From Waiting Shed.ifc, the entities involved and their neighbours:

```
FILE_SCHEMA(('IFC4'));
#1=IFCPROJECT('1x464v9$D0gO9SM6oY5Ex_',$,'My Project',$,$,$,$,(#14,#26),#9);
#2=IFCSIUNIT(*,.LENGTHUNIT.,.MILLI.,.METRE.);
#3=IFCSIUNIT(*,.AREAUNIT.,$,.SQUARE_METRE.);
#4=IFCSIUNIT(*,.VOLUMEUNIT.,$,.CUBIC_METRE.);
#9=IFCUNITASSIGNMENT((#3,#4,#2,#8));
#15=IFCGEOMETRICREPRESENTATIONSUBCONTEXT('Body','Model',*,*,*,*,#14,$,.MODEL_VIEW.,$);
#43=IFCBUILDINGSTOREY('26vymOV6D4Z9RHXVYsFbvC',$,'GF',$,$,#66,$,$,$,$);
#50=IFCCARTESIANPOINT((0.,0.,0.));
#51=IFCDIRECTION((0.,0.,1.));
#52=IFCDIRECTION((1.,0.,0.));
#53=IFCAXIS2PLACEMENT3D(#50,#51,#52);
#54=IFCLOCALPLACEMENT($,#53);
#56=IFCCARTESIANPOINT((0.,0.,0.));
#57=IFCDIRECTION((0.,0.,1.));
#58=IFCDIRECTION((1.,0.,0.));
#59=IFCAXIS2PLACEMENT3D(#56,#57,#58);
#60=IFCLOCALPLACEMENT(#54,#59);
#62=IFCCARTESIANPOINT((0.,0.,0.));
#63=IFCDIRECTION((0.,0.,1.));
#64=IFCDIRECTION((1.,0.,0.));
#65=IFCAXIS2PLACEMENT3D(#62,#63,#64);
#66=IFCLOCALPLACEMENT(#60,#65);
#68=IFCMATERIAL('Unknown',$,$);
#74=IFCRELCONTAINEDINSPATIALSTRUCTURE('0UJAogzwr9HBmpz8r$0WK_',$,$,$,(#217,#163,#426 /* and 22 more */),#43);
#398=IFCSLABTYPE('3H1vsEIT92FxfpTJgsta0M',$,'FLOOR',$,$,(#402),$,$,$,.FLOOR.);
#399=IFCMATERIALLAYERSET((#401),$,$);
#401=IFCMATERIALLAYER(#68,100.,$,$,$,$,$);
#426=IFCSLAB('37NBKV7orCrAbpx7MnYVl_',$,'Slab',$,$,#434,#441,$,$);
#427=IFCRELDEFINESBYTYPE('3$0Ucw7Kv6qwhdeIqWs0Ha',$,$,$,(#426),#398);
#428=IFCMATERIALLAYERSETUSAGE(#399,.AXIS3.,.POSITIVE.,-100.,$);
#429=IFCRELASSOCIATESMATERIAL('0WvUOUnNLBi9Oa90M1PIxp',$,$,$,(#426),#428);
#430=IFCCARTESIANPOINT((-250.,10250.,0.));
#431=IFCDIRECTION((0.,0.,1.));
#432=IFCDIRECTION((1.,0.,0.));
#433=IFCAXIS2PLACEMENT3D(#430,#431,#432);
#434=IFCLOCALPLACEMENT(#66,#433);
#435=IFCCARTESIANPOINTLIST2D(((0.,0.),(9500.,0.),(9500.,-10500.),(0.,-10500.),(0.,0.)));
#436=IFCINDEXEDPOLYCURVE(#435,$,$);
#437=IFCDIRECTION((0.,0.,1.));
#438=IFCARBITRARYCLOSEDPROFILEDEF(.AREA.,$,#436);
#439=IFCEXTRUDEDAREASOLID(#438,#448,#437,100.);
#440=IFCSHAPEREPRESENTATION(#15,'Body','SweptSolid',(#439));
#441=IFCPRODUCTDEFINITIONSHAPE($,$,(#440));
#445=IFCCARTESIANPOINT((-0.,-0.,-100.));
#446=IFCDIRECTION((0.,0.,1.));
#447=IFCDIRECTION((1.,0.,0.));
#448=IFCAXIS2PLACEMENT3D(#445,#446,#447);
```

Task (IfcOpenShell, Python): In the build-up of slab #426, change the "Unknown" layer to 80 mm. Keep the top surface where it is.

```python
import ifcopenshell
import ifcopenshell.util.element
import ifcopenshell.util.representation
import ifcopenshell.util.unit

model = ifcopenshell.open("Waiting Shed.ifc")
unit_scale = ifcopenshell.util.unit.calculate_unit_scale(model)

layer_set = model.by_id(399)
layer = next(l for l in layer_set.MaterialLayers if l.Material and l.Material.Name == "Unknown")
change = 0.08 / unit_scale - layer.LayerThickness
layer.LayerThickness += change

# Geometry does not follow the layer set by itself.
slabs = [e for e in ifcopenshell.util.element.get_elements_by_material(model, layer_set) if e.is_a("IfcSlab")]
for slab in sorted(slabs, key=lambda e: e.id()):
    body = ifcopenshell.util.representation.get_representation(slab, "Model", "Body")
    solid = body.Items[0]
    old_depth = solid.Depth
    solid.Depth += change
    # Extruded upwards: lower the start of the extrusion so the top stays.
    x, y, z = solid.Position.Location.Coordinates
    solid.Position.Location = model.createIfcCartesianPoint((x, y, z - change))
    print(slab.id(), f"{old_depth:g} -> {solid.Depth:g}")

# The layers are counted up from the underside, which has moved.
for usage in {ifcopenshell.util.element.get_material(slab) for slab in slabs}:
    usage.OffsetFromReferenceLine -= change

model.write("Waiting Shed_edited.ifc")
```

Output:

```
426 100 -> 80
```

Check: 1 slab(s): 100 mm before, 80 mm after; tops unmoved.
